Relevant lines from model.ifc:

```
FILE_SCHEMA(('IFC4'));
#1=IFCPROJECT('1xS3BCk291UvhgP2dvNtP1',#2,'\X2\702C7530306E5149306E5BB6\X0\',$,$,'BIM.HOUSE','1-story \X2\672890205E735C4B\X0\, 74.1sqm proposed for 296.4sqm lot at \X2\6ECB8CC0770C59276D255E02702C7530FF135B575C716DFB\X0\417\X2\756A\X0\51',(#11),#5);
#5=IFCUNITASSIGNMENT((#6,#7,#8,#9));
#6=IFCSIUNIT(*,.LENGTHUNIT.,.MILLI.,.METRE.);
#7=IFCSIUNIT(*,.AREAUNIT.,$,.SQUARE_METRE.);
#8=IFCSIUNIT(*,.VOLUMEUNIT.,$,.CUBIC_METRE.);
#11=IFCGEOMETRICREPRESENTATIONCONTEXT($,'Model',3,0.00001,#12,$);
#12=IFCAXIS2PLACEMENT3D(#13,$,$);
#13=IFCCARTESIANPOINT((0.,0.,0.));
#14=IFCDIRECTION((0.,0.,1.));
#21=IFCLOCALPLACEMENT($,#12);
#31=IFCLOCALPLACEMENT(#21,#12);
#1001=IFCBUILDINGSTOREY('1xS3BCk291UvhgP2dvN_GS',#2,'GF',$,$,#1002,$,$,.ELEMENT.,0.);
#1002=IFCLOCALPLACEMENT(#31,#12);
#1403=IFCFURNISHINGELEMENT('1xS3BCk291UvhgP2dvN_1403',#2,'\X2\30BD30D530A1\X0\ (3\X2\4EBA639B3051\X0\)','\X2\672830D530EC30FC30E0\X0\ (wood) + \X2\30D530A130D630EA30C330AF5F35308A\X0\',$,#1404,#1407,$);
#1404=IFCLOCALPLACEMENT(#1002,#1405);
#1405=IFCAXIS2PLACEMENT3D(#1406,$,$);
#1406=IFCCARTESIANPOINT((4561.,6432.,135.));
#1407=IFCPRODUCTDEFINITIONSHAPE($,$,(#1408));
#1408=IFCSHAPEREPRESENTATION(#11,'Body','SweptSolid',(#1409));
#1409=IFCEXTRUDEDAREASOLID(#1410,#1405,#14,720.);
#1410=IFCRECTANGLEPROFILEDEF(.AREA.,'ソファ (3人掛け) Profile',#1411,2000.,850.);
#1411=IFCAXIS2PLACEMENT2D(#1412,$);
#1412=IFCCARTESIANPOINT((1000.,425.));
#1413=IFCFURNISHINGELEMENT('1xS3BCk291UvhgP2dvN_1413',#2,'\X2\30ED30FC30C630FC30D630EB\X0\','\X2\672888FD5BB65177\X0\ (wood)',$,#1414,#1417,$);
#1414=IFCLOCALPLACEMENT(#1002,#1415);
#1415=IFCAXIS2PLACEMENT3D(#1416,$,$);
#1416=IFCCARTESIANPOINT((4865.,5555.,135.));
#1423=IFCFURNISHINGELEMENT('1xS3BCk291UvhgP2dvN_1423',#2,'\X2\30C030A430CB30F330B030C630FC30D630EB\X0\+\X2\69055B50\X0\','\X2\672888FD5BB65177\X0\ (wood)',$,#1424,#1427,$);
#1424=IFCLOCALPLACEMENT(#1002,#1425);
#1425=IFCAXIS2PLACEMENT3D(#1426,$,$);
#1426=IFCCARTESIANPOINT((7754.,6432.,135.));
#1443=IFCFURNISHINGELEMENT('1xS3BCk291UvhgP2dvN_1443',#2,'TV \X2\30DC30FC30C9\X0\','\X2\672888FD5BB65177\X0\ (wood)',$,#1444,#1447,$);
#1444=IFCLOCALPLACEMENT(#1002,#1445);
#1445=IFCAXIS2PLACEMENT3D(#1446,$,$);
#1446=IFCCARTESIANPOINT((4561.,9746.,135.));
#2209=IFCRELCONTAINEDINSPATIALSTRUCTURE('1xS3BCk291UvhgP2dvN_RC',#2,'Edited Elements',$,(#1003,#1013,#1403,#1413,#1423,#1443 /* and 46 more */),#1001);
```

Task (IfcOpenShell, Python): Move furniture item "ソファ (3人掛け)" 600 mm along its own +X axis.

```python
import ifcopenshell
import ifcopenshell.api.geometry
import ifcopenshell.util.placement
import ifcopenshell.util.unit

model = ifcopenshell.open("model.ifc")
unit_scale = ifcopenshell.util.unit.calculate_unit_scale(model)

item = model.by_guid("1xS3BCk291UvhgP2dvN_1403")
matrix = ifcopenshell.util.placement.get_local_placement(item.ObjectPlacement)
matrix[:3, 3] += matrix[:3, 0] * 0.6 / unit_scale
ifcopenshell.api.geometry.edit_object_placement(model, product=item, matrix=matrix, is_si=False)

print(ifcopenshell.util.placement.get_local_placement(item.ObjectPlacement).round(3) + 0.0)

model.write("model_v2.ifc")
```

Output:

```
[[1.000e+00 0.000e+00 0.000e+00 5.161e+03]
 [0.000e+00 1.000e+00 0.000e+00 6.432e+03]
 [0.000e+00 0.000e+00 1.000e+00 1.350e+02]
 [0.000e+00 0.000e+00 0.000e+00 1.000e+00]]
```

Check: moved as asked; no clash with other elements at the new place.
